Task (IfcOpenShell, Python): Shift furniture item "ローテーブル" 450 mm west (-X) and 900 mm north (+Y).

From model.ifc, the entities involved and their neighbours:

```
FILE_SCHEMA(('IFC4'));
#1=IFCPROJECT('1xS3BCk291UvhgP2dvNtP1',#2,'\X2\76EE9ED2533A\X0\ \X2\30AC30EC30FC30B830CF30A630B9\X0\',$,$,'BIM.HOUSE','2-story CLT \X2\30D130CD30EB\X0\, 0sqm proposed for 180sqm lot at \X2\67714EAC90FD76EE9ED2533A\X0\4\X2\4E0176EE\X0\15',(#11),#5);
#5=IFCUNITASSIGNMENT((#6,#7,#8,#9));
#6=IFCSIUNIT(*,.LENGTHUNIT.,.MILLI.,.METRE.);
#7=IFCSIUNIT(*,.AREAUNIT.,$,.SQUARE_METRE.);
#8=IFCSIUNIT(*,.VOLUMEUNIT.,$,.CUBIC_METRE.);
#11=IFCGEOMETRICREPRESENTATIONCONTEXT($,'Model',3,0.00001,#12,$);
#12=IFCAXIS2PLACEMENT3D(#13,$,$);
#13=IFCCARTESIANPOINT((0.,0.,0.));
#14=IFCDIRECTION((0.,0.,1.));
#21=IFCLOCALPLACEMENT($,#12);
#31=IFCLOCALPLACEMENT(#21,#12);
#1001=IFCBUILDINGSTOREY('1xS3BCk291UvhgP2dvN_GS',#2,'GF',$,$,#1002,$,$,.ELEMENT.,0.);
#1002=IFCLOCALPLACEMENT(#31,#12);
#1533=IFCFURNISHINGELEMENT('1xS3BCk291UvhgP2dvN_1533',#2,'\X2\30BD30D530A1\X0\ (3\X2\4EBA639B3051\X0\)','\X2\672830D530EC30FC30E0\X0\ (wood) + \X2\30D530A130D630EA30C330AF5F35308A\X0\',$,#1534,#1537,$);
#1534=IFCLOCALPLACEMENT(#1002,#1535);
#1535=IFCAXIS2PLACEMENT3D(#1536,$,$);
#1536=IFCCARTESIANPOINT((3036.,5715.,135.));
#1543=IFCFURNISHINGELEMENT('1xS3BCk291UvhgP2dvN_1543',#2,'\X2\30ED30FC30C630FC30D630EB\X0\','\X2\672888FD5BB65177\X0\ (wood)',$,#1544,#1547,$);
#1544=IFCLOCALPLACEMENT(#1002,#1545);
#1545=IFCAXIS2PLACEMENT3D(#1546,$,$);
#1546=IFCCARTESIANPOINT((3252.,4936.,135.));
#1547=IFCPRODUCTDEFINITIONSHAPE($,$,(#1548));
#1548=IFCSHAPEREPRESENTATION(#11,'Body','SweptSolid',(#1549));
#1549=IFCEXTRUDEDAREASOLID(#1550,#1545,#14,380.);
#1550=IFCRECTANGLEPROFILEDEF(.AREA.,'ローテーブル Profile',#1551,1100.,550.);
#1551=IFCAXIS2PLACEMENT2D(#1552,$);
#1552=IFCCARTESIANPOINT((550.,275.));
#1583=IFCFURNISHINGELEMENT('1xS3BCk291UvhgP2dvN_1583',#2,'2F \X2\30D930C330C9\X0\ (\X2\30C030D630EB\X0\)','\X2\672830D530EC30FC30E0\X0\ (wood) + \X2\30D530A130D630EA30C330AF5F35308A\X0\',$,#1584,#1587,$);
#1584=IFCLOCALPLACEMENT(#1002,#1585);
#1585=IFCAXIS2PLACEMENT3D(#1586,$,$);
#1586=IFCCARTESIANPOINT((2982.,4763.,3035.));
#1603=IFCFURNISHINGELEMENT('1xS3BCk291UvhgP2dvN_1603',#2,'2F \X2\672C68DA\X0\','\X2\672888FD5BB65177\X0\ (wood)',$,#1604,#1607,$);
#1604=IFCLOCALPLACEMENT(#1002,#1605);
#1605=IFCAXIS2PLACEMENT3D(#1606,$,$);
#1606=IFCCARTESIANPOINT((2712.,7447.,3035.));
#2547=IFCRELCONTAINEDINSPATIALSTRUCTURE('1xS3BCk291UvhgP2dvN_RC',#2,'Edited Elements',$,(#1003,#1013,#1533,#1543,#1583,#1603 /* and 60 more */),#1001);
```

```python
import ifcopenshell
import ifcopenshell.api.geometry
import ifcopenshell.util.placement

model = ifcopenshell.open("model.ifc")

item = model.by_guid("1xS3BCk291UvhgP2dvN_1543")
matrix = ifcopenshell.util.placement.get_local_placement(item.ObjectPlacement)
matrix[0, 3] -= 450.0
matrix[1, 3] += 900.0
ifcopenshell.api.geometry.edit_object_placement(model, product=item, matrix=matrix, is_si=False)

print(ifcopenshell.util.placement.get_local_placement(item.ObjectPlacement).round(3) + 0.0)

model.write("model-out.ifc")
```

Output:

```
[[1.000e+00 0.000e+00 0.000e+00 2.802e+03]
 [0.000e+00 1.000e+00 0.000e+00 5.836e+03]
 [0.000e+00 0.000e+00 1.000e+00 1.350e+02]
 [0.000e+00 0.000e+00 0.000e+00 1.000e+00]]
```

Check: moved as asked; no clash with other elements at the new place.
